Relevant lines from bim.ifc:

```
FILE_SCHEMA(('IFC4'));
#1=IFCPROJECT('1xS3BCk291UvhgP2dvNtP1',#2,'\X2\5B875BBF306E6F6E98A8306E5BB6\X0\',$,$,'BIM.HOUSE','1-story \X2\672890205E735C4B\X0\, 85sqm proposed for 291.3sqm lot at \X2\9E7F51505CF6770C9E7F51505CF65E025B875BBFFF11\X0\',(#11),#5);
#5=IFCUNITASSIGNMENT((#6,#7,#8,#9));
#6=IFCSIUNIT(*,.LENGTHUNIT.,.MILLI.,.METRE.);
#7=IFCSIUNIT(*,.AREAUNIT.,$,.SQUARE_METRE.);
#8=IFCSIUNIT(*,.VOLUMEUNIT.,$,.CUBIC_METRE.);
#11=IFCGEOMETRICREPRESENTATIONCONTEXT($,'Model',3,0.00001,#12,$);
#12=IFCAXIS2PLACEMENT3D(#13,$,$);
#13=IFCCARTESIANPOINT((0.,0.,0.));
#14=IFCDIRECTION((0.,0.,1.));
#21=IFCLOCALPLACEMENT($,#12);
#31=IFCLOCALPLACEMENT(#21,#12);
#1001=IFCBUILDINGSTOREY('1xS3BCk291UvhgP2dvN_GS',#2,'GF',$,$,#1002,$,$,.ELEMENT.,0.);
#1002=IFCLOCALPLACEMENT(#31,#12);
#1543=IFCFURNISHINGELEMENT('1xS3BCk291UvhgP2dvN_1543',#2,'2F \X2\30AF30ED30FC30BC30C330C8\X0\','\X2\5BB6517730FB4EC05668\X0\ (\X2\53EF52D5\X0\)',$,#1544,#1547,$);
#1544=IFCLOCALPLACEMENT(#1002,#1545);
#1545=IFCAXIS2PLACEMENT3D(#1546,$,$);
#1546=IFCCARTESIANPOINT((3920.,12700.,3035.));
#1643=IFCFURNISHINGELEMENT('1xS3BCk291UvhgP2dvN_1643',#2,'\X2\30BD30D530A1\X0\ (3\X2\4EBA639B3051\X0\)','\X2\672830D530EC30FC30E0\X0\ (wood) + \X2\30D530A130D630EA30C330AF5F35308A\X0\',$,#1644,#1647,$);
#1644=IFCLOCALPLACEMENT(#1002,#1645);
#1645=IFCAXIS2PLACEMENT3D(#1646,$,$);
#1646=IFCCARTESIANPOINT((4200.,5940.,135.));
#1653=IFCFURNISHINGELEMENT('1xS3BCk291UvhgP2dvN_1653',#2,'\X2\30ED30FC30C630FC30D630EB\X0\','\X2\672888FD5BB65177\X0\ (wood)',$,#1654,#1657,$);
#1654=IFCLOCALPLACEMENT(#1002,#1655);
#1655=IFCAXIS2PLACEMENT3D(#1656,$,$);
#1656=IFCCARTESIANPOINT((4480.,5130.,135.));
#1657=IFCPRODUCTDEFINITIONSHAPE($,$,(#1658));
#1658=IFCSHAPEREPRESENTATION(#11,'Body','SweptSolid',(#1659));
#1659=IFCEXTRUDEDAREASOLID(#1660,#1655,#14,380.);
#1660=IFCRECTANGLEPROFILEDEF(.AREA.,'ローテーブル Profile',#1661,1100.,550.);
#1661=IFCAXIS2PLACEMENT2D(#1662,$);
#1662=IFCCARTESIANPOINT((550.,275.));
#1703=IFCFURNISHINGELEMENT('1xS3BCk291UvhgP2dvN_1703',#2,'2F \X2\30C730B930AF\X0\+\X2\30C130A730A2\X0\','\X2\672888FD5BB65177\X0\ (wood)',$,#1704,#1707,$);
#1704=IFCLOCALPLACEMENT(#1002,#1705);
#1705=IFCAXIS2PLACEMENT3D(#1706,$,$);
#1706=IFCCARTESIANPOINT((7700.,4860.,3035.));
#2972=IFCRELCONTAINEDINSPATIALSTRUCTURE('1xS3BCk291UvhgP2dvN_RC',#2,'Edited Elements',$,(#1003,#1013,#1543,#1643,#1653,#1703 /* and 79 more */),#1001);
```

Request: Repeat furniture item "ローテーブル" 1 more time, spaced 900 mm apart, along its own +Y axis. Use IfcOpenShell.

```python
import ifcopenshell
import ifcopenshell.api.geometry
import ifcopenshell.api.root
import ifcopenshell.util.element
import ifcopenshell.util.placement
import ifcopenshell.util.unit

model = ifcopenshell.open("bim.ifc")
unit_scale = ifcopenshell.util.unit.calculate_unit_scale(model)


def reuse_history(source, copy):
    """copy_class also copies each property set's owner history, people and application; keep the originals."""
    for rel in copy.IsDefinedBy:
        if rel.is_a("IfcRelDefinesByProperties") and (history := rel.RelatingPropertyDefinition.OwnerHistory):
            rel.RelatingPropertyDefinition.OwnerHistory = source.OwnerHistory
            ifcopenshell.util.element.remove_deep2(model, history)


source = model.by_id(1653)
base = ifcopenshell.util.placement.get_local_placement(source.ObjectPlacement)
step = base[:3, 1] * 0.9 / unit_scale

for i in range(1, 2):
    copy = ifcopenshell.api.root.copy_class(model, product=source)
    copy.Representation = ifcopenshell.util.element.copy_deep(
        model, source.Representation, exclude=["IfcGeometricRepresentationContext", "IfcRepresentationMap"]
    )
    reuse_history(source, copy)
    matrix = base.copy()
    matrix[:3, 3] += i * step
    print("added at", matrix[:3, 3].round(3) + 0.0)
    ifcopenshell.api.geometry.edit_object_placement(model, product=copy, matrix=matrix, is_si=False)

model.write("bim_edited.ifc")
```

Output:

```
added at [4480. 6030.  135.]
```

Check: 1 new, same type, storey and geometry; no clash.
